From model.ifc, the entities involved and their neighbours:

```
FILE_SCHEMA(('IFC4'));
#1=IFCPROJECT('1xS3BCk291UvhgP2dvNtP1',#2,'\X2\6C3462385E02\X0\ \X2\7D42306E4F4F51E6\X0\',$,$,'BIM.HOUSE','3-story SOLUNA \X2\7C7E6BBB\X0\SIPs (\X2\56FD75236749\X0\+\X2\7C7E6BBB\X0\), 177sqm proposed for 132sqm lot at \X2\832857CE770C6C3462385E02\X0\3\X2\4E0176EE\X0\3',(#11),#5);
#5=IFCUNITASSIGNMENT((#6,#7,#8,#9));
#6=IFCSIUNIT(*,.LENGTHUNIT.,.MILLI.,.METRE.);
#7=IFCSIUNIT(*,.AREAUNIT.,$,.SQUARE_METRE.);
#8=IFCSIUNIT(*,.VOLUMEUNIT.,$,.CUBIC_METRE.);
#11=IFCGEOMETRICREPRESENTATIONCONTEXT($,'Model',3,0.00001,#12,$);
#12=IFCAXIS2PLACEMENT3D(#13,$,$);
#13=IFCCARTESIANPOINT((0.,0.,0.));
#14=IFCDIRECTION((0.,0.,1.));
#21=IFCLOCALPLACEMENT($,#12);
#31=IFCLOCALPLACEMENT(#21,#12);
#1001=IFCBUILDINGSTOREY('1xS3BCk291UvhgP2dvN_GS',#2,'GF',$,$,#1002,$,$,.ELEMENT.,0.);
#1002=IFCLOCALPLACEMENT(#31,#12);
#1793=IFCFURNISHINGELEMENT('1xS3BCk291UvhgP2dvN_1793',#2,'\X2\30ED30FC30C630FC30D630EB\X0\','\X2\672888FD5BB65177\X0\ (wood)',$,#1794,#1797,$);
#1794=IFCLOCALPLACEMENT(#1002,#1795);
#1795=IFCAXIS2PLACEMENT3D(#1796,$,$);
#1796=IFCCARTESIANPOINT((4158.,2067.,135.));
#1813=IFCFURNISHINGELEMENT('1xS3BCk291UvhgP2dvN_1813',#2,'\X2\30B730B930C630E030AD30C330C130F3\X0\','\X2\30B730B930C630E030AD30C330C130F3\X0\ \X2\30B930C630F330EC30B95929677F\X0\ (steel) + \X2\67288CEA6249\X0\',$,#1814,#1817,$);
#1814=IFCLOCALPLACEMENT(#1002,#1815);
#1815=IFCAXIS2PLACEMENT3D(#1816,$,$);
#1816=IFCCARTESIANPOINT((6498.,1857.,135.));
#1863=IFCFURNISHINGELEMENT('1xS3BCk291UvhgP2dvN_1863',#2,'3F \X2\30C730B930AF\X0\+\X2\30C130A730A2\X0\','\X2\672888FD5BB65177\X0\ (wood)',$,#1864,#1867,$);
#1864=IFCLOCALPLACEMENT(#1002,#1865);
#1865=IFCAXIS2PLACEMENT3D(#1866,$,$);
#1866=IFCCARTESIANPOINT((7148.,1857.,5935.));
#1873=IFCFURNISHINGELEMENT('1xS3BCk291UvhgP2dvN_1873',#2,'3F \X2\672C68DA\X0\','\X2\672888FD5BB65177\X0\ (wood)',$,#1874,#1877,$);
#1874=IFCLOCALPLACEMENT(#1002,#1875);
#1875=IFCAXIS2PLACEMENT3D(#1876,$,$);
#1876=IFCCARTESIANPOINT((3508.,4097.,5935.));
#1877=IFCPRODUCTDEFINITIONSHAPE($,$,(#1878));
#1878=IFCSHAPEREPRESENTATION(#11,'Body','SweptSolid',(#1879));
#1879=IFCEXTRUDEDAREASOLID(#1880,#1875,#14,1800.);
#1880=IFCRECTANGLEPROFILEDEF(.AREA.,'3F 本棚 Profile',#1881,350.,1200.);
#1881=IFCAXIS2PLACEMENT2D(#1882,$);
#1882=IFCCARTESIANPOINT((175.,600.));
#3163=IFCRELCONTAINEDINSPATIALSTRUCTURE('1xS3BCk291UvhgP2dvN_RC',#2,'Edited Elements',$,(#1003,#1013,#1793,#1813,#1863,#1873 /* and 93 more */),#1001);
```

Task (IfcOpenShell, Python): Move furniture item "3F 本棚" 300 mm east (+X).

```python
import ifcopenshell
import ifcopenshell.api.geometry
import ifcopenshell.util.placement

model = ifcopenshell.open("model.ifc")

item = model.by_guid("1xS3BCk291UvhgP2dvN_1873")
matrix = ifcopenshell.util.placement.get_local_placement(item.ObjectPlacement)
matrix[0, 3] += 300.0
ifcopenshell.api.geometry.edit_object_placement(model, product=item, matrix=matrix, is_si=False)

print(ifcopenshell.util.placement.get_local_placement(item.ObjectPlacement).round(3) + 0.0)

model.write("model-out.ifc")
```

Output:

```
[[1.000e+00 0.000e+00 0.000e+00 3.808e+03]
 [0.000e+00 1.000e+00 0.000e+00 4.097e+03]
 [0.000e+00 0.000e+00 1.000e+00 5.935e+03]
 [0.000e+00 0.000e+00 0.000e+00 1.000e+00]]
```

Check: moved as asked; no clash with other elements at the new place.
